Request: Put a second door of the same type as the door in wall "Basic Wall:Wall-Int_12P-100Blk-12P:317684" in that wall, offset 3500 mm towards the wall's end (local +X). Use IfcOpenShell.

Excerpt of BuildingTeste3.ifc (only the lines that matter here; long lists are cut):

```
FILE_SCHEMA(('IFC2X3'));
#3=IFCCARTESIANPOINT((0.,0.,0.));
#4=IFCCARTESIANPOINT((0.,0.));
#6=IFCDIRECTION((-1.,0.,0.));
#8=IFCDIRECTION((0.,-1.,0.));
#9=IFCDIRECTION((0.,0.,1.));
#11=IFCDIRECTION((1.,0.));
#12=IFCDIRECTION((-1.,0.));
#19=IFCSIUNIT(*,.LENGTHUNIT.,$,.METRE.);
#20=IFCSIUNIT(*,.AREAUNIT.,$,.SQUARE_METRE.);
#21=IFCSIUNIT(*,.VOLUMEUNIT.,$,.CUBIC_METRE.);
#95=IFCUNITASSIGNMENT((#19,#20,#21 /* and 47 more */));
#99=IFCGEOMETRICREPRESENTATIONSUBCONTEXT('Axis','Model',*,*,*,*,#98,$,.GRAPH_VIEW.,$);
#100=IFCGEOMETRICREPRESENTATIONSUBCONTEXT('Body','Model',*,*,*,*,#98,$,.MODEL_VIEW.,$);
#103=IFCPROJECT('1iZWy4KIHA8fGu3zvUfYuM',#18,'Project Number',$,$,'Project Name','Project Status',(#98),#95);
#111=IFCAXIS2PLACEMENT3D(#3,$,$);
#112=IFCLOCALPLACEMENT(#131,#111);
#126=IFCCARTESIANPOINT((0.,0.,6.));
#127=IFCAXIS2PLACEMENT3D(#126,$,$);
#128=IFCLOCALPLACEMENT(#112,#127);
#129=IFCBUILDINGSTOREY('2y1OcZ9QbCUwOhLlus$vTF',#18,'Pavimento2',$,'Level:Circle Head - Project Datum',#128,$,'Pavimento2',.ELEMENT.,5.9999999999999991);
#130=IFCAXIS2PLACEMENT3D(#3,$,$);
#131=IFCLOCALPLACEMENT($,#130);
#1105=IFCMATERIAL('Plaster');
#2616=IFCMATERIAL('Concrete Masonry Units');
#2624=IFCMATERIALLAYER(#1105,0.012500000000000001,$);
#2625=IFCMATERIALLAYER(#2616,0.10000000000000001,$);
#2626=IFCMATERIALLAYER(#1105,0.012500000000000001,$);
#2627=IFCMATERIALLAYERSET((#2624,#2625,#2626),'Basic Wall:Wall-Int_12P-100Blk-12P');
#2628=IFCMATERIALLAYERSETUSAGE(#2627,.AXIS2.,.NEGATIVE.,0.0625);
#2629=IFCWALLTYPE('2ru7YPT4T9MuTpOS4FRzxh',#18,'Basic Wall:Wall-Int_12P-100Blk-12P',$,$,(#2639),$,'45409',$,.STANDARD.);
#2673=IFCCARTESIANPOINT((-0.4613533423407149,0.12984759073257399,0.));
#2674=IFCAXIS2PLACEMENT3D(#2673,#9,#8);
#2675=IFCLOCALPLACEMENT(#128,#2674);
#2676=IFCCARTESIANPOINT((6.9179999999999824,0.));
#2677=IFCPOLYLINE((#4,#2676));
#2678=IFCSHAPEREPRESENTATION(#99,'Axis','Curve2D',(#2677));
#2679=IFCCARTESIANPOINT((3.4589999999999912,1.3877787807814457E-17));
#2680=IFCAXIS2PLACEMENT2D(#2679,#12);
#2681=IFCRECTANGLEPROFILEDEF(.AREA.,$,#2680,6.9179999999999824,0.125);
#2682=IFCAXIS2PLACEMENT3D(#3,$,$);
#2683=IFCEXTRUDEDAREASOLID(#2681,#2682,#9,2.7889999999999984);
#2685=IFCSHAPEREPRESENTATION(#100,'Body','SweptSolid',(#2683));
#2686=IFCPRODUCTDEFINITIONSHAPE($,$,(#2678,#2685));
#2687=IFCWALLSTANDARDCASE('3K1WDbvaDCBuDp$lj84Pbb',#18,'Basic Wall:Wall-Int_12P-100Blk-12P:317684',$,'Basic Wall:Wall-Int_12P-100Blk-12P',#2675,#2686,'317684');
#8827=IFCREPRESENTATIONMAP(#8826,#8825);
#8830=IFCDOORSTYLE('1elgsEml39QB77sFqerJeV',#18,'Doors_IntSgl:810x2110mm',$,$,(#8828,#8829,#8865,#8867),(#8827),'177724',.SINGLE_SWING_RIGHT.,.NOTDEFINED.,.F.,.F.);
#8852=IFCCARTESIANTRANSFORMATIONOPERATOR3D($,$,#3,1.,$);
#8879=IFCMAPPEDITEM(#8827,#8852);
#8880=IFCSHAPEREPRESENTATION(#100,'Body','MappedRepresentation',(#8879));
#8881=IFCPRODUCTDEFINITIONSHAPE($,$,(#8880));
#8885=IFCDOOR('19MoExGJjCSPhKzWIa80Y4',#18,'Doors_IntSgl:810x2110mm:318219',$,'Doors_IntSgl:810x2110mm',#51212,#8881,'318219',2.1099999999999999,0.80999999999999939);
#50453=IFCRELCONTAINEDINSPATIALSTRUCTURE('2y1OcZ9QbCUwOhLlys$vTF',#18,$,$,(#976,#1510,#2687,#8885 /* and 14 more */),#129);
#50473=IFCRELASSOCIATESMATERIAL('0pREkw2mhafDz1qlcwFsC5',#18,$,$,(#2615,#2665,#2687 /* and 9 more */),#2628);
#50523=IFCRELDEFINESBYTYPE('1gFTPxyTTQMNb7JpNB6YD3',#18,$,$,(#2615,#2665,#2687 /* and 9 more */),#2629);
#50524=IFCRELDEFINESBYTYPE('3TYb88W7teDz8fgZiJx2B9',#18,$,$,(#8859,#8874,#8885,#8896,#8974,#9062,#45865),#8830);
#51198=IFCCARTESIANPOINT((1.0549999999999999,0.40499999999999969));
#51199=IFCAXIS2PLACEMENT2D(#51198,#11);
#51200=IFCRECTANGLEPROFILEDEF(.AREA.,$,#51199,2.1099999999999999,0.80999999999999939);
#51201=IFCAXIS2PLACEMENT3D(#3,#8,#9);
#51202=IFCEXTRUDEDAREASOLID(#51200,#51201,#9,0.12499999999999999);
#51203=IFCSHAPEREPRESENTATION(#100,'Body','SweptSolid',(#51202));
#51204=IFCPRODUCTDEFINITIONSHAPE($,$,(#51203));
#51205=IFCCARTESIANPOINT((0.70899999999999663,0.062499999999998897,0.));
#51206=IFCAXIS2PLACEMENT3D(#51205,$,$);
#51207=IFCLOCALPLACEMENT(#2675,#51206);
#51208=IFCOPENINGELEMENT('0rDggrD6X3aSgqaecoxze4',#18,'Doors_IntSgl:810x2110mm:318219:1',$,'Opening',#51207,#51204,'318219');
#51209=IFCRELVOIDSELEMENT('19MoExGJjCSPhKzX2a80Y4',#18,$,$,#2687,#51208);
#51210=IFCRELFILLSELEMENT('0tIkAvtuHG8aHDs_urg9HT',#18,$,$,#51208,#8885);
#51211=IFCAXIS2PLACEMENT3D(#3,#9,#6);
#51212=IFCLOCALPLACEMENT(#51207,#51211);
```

```python
import ifcopenshell
import ifcopenshell.api.feature
import ifcopenshell.api.geometry
import ifcopenshell.api.root
import ifcopenshell.geom
import ifcopenshell.util.element
import ifcopenshell.util.placement
import ifcopenshell.util.shape
import ifcopenshell.util.unit

model = ifcopenshell.open("BuildingTeste3.ifc")
unit_scale = ifcopenshell.util.unit.calculate_unit_scale(model)
settings = ifcopenshell.geom.settings()


def volume(element):
    """Net volume in cubic metres, openings subtracted."""
    shape = ifcopenshell.geom.create_shape(settings, element)
    return ifcopenshell.util.shape.get_volume(shape.geometry)


def reuse_history(source, copy):
    """copy_class also copies each property set's owner history, people and application; keep the originals."""
    for rel in copy.IsDefinedBy:
        if rel.is_a("IfcRelDefinesByProperties") and (history := rel.RelatingPropertyDefinition.OwnerHistory):
            rel.RelatingPropertyDefinition.OwnerHistory = source.OwnerHistory
            ifcopenshell.util.element.remove_deep2(model, history)


door = model.by_guid("19MoExGJjCSPhKzWIa80Y4")
opening = door.FillsVoids[0].RelatingOpeningElement
wall = opening.VoidsElements[0].RelatingBuildingElement
before = volume(wall)
shift = ifcopenshell.util.placement.get_local_placement(wall.ObjectPlacement)[:3, 0] * 3.5 / unit_scale

# copy_class copies the void relationship, type, container and properties, but no geometry.
new_opening = ifcopenshell.api.root.copy_class(model, product=opening)
new_opening.Representation = ifcopenshell.util.element.copy_deep(
    model, opening.Representation, exclude=["IfcGeometricRepresentationContext", "IfcRepresentationMap"]
)
new_opening.Name = "Doors_IntSgl:810x2110mm"
new_opening.Tag = None
new_door = ifcopenshell.api.root.copy_class(model, product=door)
new_door.Representation = ifcopenshell.util.element.copy_deep(
    model, door.Representation, exclude=["IfcGeometricRepresentationContext", "IfcRepresentationMap"]
)
new_door.Name = "Doors_IntSgl:810x2110mm"
new_door.Tag = None
reuse_history(door, new_door)
fills = ifcopenshell.api.feature.add_filling(model, opening=new_opening, element=new_door)
fills.OwnerHistory = new_door.OwnerHistory  # required in IFC2X3

for old, new in ((opening, new_opening), (door, new_door)):
    matrix = ifcopenshell.util.placement.get_local_placement(old.ObjectPlacement)
    matrix[:3, 3] += shift
    ifcopenshell.api.geometry.edit_object_placement(model, product=new, matrix=matrix, is_si=False)

after = volume(wall)

print(f"wall volume {before:.3f} -> {after:.3f} m3")

model.write("BuildingTeste3_rev.ifc")
```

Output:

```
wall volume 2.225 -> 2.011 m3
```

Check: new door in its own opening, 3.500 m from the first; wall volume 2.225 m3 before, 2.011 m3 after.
